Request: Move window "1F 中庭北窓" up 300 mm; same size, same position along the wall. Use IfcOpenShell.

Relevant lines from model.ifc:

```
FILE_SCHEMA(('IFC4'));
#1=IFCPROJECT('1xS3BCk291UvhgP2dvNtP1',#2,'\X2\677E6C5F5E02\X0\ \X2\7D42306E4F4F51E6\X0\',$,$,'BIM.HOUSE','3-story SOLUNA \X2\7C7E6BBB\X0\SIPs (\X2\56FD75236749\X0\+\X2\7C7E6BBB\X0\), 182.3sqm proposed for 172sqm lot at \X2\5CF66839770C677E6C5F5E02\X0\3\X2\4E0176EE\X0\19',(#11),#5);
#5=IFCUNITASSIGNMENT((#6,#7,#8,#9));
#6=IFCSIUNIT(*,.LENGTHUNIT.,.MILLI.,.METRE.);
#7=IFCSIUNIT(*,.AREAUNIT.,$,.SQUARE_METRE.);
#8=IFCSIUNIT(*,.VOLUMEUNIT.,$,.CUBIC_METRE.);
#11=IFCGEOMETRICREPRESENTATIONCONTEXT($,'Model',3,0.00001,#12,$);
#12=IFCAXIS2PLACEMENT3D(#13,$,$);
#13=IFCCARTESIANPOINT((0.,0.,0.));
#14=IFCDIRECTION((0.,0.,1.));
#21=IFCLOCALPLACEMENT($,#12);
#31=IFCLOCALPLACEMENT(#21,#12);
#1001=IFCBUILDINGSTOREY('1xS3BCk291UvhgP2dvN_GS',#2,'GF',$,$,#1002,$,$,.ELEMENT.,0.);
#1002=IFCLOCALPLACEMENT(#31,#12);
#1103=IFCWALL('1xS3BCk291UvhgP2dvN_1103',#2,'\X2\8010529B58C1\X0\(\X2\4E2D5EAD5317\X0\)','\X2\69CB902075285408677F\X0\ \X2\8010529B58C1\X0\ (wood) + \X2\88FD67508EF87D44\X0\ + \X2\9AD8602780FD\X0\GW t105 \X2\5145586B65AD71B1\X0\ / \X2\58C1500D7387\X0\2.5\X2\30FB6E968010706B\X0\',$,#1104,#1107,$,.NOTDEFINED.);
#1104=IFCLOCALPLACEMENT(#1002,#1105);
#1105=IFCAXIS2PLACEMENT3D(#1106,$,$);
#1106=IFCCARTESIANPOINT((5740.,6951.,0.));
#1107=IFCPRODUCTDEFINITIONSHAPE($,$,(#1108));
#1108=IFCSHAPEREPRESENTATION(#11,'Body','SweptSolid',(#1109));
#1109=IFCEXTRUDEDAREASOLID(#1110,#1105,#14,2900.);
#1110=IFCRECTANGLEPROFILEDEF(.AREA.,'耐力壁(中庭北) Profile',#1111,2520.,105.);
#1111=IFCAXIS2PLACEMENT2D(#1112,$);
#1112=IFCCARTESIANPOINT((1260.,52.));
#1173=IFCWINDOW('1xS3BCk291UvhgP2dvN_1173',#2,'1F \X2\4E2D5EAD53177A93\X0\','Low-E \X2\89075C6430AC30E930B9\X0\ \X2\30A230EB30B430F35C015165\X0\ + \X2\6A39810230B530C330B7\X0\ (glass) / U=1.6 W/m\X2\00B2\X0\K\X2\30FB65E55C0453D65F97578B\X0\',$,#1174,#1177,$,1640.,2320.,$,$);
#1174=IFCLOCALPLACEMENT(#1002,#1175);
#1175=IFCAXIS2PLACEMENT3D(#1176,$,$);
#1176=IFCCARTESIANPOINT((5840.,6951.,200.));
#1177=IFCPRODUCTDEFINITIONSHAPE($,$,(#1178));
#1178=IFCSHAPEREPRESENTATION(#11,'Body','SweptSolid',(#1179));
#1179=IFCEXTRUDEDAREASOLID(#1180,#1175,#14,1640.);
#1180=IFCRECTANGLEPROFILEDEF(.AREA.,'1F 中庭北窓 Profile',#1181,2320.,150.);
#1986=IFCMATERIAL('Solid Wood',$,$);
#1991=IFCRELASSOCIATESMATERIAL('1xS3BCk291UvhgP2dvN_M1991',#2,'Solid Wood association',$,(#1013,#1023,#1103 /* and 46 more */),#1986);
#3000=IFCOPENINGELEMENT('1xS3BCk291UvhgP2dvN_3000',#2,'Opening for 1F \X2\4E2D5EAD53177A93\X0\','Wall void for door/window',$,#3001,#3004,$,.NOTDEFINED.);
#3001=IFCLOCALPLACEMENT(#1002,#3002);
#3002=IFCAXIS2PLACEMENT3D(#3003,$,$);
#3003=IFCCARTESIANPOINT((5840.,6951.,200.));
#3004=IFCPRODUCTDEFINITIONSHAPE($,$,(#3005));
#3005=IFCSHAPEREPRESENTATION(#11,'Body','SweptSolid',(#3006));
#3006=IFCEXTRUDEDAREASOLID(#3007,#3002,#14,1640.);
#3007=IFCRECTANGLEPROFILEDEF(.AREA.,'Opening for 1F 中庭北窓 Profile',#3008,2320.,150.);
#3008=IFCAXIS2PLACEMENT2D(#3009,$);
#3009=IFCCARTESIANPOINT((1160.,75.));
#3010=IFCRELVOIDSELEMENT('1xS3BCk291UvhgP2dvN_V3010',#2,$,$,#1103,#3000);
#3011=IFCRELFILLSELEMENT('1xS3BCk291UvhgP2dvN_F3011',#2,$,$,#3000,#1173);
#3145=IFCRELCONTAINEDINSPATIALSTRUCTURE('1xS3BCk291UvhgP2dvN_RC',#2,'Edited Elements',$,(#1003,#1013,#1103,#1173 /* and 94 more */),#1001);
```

```python
import numpy as np
import ifcopenshell
import ifcopenshell.api.geometry
import ifcopenshell.util.placement
import ifcopenshell.util.unit

model = ifcopenshell.open("model.ifc")
unit_scale = ifcopenshell.util.unit.calculate_unit_scale(model)

window = model.by_guid("1xS3BCk291UvhgP2dvN_1173")
opening = window.FillsVoids[0].RelatingOpeningElement
dz = 0.3 / unit_scale

shift = np.array([0.0, 0.0, dz])
# The window is not placed relative to its opening, so move both.
for product in (opening, window):
    matrix = ifcopenshell.util.placement.get_local_placement(product.ObjectPlacement)
    matrix[:3, 3] += shift
    ifcopenshell.api.geometry.edit_object_placement(model, product=product, matrix=matrix, is_si=False)

print(f"moved by {dz * unit_scale:+.3f} m")

model.write("model_rev.ifc")
```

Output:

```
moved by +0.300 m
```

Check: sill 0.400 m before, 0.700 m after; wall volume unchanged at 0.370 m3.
